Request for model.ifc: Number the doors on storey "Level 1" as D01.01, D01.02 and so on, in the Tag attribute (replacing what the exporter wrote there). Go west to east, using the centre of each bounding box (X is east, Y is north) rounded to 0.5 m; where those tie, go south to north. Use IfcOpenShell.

First a look at what the model holds.

```python
import ifcopenshell
import ifcopenshell.util.element
import ifcopenshell.util.placement

model = ifcopenshell.open("model.ifc")
print(model.schema)
storey = next(s for s in model.by_type("IfcBuildingStorey") if s.Name == "Level 1")
doors = [e for e in ifcopenshell.util.element.get_decomposition(storey) if e.is_a("IfcDoor")]
for e in sorted(doors, key=lambda e: e.id()):
    origin = ifcopenshell.util.placement.get_local_placement(e.ObjectPlacement)[:3, 3]
    print(e.id(), e.Tag, e.Name, origin.round(2) + 0.0, sep=" | ")
```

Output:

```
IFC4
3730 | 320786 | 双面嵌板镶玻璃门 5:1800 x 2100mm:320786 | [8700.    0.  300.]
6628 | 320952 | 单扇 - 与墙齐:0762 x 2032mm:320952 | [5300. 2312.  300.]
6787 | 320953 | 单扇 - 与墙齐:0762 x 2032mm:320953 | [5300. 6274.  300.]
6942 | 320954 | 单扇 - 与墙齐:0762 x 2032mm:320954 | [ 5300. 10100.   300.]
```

```python
import ifcopenshell
import ifcopenshell.geom
import ifcopenshell.util.element
import ifcopenshell.util.shape

model = ifcopenshell.open("model.ifc")
settings = ifcopenshell.geom.settings()
settings.set("use-world-coords", True)


def centre(element):
    shape = ifcopenshell.geom.create_shape(settings, element)
    return ifcopenshell.util.shape.get_bbox_centroid(shape.geometry)


storey = next(s for s in model.by_type("IfcBuildingStorey") if s.Name == "Level 1")
doors = [e for e in ifcopenshell.util.element.get_decomposition(storey) if e.is_a("IfcDoor")]

# Insertion points can sit at a corner or the storey origin, so sort by the geometry (in metres).
centres = {e: centre(e) for e in doors}
doors.sort(key=lambda e: (round(centres[e][0] / 0.5), centres[e][1]))

for i, e in enumerate(doors, start=1):
    number = f"D01.{i:02d}"
    e.Tag = number
    print(e.id(), number)

model.write("model_edited.ifc")
```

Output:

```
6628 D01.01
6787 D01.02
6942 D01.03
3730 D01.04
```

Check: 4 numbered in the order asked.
